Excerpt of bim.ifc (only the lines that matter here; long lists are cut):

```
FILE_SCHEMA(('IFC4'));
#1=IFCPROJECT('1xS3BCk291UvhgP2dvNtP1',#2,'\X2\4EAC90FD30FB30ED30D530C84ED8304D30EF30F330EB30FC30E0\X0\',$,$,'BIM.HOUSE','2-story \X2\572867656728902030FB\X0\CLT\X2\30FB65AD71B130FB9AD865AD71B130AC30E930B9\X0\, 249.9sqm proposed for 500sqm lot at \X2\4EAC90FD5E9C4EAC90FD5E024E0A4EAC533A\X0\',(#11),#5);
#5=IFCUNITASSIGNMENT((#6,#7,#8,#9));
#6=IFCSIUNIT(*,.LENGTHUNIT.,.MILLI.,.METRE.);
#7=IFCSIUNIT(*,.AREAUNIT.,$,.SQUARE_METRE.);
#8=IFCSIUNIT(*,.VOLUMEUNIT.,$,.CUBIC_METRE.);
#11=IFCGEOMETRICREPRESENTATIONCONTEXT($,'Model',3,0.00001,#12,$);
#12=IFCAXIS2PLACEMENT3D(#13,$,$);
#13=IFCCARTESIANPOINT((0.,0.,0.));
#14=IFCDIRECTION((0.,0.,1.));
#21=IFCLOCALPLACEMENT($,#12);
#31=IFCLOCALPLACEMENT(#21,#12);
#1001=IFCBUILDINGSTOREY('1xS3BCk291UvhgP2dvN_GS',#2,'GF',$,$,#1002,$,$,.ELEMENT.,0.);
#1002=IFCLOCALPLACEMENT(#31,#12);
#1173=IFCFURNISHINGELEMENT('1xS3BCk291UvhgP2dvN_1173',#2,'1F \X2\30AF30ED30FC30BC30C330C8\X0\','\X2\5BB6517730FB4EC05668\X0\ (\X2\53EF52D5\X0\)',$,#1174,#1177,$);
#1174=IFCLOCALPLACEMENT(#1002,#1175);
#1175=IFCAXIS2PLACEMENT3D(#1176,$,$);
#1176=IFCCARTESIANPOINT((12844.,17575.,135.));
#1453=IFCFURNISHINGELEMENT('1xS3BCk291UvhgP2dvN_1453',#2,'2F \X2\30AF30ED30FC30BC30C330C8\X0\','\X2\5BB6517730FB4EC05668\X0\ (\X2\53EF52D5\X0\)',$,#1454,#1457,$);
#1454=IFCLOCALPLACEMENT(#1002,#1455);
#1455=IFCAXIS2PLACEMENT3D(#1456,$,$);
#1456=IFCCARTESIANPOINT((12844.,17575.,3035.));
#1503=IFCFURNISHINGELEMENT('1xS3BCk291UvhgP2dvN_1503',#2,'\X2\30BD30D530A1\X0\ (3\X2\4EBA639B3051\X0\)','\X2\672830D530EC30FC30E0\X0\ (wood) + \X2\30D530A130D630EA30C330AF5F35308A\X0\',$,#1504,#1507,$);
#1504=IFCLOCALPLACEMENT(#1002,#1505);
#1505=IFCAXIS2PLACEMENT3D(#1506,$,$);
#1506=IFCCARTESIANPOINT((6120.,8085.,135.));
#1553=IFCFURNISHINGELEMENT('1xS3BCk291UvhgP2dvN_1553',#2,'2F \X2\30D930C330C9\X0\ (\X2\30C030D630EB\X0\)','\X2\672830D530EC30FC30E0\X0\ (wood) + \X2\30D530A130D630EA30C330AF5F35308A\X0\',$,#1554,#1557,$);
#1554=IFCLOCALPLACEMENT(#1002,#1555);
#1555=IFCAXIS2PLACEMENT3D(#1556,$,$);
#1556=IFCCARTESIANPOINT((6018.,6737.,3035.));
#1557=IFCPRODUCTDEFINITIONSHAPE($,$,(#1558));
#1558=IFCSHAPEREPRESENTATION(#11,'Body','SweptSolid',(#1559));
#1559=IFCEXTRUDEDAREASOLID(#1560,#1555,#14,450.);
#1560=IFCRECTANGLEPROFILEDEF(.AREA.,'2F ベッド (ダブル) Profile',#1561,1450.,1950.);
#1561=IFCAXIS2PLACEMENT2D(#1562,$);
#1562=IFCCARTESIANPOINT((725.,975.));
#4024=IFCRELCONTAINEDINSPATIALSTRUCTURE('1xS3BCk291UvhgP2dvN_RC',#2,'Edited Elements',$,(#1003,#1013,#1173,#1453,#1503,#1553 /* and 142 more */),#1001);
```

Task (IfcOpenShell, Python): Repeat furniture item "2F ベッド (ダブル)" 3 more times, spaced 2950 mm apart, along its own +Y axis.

```python
import ifcopenshell
import ifcopenshell.api.geometry
import ifcopenshell.api.root
import ifcopenshell.util.element
import ifcopenshell.util.placement
import ifcopenshell.util.unit

model = ifcopenshell.open("bim.ifc")
unit_scale = ifcopenshell.util.unit.calculate_unit_scale(model)


def reuse_history(source, copy):
    """copy_class also copies each property set's owner history, people and application; keep the originals."""
    for rel in copy.IsDefinedBy:
        if rel.is_a("IfcRelDefinesByProperties") and (history := rel.RelatingPropertyDefinition.OwnerHistory):
            rel.RelatingPropertyDefinition.OwnerHistory = source.OwnerHistory
            ifcopenshell.util.element.remove_deep2(model, history)


source = model.by_guid("1xS3BCk291UvhgP2dvN_1553")
base = ifcopenshell.util.placement.get_local_placement(source.ObjectPlacement)
step = base[:3, 1] * 2.95 / unit_scale

for i in range(1, 4):
    copy = ifcopenshell.api.root.copy_class(model, product=source)
    copy.Representation = ifcopenshell.util.element.copy_deep(
        model, source.Representation, exclude=["IfcGeometricRepresentationContext", "IfcRepresentationMap"]
    )
    reuse_history(source, copy)
    matrix = base.copy()
    matrix[:3, 3] += i * step
    print("added at", matrix[:3, 3].round(3) + 0.0)
    ifcopenshell.api.geometry.edit_object_placement(model, product=copy, matrix=matrix, is_si=False)

model.write("bim_updated.ifc")
```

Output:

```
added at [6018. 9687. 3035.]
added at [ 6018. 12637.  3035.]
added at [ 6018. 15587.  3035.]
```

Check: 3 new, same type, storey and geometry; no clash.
